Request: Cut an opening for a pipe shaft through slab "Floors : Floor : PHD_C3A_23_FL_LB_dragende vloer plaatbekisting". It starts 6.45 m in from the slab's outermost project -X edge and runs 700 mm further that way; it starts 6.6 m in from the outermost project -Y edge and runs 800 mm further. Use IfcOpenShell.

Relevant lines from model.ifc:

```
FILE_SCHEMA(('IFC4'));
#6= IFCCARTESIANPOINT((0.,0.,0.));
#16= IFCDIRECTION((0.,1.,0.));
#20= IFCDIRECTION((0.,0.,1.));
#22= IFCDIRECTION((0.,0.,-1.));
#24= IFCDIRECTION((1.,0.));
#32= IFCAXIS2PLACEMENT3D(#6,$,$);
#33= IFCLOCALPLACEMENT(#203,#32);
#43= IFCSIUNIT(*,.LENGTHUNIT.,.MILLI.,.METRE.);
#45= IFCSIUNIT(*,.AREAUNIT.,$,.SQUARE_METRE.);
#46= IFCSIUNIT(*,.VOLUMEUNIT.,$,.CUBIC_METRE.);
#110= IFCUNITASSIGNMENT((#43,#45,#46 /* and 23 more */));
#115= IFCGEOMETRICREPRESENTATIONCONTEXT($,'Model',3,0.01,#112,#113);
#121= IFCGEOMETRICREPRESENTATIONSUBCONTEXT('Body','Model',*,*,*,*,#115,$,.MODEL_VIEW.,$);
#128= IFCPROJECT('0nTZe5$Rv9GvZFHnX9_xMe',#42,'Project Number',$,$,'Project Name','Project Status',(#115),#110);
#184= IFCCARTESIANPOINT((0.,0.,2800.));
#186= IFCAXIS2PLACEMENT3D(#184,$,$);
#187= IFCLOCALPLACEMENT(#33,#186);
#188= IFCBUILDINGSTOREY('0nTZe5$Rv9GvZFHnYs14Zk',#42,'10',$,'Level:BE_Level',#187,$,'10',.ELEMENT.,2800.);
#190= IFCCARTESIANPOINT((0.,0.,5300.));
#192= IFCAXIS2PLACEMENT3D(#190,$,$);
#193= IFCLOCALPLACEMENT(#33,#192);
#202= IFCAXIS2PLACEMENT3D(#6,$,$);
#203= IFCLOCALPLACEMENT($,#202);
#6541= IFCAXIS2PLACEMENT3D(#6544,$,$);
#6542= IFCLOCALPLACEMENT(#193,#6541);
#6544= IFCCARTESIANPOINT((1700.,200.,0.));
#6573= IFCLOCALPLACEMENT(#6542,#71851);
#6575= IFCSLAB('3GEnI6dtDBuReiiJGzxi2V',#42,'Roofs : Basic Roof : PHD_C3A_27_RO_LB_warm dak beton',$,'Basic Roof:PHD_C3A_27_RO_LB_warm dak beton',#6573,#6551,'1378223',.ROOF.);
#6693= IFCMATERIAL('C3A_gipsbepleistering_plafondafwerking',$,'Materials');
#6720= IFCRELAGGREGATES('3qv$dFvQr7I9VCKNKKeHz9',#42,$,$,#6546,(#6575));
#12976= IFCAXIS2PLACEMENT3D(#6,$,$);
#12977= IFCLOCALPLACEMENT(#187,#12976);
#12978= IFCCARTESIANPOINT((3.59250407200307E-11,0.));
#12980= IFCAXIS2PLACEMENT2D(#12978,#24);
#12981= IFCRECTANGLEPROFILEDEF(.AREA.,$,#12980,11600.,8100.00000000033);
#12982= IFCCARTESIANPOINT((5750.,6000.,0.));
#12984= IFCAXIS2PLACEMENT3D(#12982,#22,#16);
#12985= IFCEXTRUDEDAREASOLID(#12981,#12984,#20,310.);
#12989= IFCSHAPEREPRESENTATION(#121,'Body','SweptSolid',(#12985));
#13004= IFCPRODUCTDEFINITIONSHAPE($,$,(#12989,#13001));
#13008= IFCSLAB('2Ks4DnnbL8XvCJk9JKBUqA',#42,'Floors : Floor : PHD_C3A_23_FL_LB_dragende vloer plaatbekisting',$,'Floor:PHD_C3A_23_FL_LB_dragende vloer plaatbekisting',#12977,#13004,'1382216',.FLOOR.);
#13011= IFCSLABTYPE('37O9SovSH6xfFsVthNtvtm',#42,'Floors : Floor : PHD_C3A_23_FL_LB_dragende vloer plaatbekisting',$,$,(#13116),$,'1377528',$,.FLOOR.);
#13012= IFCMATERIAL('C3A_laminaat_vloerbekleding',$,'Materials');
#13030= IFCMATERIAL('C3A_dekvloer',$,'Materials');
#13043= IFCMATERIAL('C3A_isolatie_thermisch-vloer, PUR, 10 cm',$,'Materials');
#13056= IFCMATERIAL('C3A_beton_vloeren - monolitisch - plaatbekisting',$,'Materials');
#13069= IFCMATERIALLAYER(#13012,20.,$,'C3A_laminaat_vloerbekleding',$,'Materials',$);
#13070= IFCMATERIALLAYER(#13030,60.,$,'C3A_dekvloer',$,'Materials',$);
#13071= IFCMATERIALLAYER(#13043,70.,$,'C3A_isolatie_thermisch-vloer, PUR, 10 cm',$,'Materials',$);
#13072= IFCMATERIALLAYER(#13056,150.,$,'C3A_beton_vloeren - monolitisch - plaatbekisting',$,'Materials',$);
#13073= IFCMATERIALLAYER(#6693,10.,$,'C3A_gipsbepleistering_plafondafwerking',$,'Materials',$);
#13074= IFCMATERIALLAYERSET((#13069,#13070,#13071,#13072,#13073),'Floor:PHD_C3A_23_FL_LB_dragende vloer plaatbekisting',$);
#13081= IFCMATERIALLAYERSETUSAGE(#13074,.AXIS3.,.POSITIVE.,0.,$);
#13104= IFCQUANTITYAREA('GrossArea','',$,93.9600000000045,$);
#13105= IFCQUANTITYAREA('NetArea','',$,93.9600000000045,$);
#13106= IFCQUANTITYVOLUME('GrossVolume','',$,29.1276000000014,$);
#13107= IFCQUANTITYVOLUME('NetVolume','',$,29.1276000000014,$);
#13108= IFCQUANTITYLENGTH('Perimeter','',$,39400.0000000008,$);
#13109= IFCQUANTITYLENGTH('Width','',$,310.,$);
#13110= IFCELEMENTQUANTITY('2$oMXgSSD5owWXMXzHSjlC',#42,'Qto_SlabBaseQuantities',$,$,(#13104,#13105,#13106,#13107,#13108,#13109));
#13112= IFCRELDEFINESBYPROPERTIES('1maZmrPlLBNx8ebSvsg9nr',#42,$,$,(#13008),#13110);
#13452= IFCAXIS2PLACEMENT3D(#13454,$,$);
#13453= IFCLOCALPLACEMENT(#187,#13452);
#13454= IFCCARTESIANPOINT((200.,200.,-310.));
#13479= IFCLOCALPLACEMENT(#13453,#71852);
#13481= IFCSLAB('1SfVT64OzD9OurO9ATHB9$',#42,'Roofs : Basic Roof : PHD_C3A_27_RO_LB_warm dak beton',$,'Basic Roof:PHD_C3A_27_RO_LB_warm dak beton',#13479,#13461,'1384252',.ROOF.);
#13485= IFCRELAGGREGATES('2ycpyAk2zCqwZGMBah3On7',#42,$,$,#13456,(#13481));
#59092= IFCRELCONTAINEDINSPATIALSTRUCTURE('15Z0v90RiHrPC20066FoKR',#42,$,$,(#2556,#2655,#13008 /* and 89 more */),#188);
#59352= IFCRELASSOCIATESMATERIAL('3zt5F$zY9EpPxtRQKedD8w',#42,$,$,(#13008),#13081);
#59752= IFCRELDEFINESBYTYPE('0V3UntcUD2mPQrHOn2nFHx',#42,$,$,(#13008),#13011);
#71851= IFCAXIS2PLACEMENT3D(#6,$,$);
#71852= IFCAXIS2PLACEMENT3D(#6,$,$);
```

```python
import numpy as np
import ifcopenshell
import ifcopenshell.api.feature
import ifcopenshell.api.geometry
import ifcopenshell.api.pset
import ifcopenshell.api.root
import ifcopenshell.geom
import ifcopenshell.util.element
import ifcopenshell.util.placement
import ifcopenshell.util.representation
import ifcopenshell.util.shape
import ifcopenshell.util.unit

model = ifcopenshell.open("model.ifc")
unit_scale = ifcopenshell.util.unit.calculate_unit_scale(model)
area_scale = ifcopenshell.util.unit.calculate_unit_scale(model, "AREAUNIT")
volume_scale = ifcopenshell.util.unit.calculate_unit_scale(model, "VOLUMEUNIT")
settings = ifcopenshell.geom.settings()


def volume(element):
    """Net volume in cubic metres, openings subtracted."""
    shape = ifcopenshell.geom.create_shape(settings, element)
    return ifcopenshell.util.shape.get_volume(shape.geometry)


slab = model.by_id(13008)
before = volume(slab)

# Extent in the slab's own axes, in metres. The edges named are its -X and -Y sides.
slab_shape = ifcopenshell.geom.create_shape(settings, slab)
vertices = ifcopenshell.util.shape.get_vertices(slab_shape.geometry)
x_min, y_min, bottom = vertices.min(axis=0)
top = vertices[:, 2].max()

opening = ifcopenshell.api.root.create_entity(model, ifc_class="IfcOpeningElement", name="Pipe shaft opening", predefined_type="OPENING")
context = ifcopenshell.util.representation.get_context(model, "Model", "Body", "MODEL_VIEW")
width, depth = 0.7, 0.8
outline = [(0.0, 0.0), (width, 0.0), (width, depth), (0.0, depth), (0.0, 0.0)]
# Overshoot both faces by 50 mm so the cut is clean.
shape = ifcopenshell.api.geometry.add_slab_representation(
    model, context=context, depth=top - bottom + 0.1, polyline=outline
)
ifcopenshell.api.geometry.assign_representation(model, product=opening, representation=shape)

matrix = ifcopenshell.util.placement.get_local_placement(slab.ObjectPlacement)
matrix[:, 3] = matrix @ np.append(np.array([x_min + 6.45, y_min + 6.6, bottom - 0.05]) / unit_scale, 1.0)
ifcopenshell.api.geometry.edit_object_placement(model, product=opening, matrix=matrix, is_si=False)
ifcopenshell.api.feature.add_feature(model, feature=opening, element=slab)

after = volume(slab)

# Update the slab's stored quantities.
qto = model.by_id(ifcopenshell.util.element.get_pset(slab, "Qto_SlabBaseQuantities", should_inherit=False)["id"])
ifcopenshell.api.pset.edit_qto(model, qto=qto, properties={
    "NetArea": after / (top - bottom) / area_scale,
    "NetVolume": after / volume_scale,
})

print(f"slab volume {before:.3f} -> {after:.3f} m3")

model.write("model-out.ifc")
```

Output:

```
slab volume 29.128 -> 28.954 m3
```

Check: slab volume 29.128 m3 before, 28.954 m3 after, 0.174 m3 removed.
